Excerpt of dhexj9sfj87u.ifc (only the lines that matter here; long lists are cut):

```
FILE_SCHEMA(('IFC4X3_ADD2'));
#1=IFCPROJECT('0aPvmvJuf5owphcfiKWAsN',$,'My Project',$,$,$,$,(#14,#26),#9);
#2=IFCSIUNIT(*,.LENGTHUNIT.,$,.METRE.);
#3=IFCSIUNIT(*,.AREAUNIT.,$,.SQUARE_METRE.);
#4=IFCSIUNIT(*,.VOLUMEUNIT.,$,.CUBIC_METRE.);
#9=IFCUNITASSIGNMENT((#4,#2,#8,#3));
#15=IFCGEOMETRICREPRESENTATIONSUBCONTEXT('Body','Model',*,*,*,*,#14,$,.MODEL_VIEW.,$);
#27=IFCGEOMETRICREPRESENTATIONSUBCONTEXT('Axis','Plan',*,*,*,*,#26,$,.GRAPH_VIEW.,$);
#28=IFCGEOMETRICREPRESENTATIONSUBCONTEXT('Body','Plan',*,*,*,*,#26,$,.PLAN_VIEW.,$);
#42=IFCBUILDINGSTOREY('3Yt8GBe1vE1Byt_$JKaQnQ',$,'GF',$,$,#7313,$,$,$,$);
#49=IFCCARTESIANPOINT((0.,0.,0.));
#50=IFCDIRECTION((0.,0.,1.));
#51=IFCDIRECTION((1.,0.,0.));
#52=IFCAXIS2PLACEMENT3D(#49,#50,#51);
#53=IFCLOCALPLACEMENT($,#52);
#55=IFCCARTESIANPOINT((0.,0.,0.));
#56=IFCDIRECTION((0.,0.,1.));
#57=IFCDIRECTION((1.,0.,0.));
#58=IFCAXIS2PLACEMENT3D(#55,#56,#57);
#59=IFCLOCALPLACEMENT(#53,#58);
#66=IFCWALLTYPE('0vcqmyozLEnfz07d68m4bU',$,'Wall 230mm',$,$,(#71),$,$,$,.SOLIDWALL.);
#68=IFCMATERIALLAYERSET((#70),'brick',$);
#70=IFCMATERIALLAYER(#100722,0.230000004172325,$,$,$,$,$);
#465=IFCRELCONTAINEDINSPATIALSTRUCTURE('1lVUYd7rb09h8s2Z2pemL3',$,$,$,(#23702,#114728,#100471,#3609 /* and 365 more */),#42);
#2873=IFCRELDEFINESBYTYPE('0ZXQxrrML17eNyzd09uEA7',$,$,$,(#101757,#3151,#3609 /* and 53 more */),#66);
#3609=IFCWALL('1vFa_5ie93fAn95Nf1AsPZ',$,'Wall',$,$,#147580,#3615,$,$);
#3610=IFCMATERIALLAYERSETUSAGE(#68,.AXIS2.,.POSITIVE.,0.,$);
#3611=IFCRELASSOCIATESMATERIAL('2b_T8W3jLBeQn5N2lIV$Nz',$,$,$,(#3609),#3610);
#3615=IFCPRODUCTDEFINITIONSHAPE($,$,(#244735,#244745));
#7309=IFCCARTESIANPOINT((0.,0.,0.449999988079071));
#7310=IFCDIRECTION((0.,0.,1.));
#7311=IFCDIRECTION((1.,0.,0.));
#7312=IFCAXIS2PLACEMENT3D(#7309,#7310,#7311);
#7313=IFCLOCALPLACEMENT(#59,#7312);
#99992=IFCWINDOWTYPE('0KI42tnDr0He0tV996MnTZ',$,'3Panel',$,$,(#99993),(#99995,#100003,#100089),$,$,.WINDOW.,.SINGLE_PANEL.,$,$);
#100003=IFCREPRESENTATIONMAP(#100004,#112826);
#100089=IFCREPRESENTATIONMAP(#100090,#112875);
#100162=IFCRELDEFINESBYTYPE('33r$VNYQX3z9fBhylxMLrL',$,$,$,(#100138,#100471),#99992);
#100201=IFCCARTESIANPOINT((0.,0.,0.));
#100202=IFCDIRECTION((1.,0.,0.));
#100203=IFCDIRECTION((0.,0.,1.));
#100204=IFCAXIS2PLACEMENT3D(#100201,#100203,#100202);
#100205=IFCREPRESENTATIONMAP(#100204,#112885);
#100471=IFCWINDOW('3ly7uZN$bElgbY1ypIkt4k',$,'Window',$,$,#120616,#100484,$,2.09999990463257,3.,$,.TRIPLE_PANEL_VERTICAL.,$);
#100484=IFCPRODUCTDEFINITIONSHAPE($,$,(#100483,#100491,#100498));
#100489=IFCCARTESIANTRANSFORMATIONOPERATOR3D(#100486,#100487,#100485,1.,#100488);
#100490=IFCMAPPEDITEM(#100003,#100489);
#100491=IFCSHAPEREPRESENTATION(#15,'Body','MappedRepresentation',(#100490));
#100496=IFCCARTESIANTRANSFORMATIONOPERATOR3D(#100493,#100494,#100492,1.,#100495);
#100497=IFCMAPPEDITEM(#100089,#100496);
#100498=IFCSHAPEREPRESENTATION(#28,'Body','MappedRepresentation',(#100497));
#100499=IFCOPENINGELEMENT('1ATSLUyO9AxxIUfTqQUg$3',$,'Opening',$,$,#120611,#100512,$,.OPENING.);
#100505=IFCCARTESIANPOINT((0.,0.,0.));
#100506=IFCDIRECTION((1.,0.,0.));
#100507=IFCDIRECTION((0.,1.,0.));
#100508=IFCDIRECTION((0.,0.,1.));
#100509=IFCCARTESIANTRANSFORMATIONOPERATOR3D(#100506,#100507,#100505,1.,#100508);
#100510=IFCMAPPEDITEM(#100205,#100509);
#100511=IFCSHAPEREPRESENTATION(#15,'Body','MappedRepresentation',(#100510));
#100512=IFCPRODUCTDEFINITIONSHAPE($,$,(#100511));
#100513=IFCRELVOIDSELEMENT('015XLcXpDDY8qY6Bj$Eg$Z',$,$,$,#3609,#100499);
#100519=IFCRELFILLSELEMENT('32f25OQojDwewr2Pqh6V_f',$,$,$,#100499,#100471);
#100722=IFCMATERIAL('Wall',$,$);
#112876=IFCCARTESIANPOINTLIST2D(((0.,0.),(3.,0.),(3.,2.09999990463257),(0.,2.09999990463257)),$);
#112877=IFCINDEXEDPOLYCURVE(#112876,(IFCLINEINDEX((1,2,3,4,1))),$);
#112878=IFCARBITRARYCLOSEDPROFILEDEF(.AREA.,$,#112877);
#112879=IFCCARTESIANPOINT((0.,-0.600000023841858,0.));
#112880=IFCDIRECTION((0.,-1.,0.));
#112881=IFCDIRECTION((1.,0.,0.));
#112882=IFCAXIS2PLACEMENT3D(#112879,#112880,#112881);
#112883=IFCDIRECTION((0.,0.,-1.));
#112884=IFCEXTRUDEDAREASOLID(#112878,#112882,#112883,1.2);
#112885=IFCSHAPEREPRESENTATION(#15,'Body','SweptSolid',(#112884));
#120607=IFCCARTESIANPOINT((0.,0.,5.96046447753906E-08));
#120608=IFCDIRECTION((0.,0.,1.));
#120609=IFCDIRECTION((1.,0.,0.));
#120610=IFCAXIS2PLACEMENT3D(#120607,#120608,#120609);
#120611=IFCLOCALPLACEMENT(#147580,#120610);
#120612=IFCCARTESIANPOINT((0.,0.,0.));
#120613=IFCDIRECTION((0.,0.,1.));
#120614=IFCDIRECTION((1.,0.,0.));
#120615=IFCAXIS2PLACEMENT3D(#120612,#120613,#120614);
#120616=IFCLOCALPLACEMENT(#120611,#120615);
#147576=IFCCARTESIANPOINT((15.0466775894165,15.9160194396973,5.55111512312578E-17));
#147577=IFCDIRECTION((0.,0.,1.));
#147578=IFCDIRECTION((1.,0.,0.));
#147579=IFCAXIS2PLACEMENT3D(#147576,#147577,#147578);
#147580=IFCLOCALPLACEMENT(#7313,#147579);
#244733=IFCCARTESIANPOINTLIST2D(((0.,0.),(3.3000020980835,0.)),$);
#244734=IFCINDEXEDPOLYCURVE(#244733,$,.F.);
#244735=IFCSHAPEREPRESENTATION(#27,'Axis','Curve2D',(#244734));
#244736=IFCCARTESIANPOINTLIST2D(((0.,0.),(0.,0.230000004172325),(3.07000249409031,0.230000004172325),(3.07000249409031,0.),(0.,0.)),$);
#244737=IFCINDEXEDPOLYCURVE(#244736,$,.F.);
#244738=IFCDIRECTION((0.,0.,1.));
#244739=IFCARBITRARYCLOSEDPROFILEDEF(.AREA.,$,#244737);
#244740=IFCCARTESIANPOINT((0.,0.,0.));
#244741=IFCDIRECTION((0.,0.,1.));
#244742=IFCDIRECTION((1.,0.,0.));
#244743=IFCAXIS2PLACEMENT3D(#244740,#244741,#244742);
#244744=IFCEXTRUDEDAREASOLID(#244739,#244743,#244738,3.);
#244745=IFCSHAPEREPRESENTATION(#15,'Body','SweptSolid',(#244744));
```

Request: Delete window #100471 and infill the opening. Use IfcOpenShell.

```python
import ifcopenshell
import ifcopenshell.api.feature
import ifcopenshell.api.root
import ifcopenshell.geom
import ifcopenshell.util.shape

model = ifcopenshell.open("dhexj9sfj87u.ifc")
settings = ifcopenshell.geom.settings()


def volume(element):
    """Net volume in cubic metres, openings subtracted."""
    shape = ifcopenshell.geom.create_shape(settings, element)
    return ifcopenshell.util.shape.get_volume(shape.geometry)


window = model.by_id(100471)
opening = window.FillsVoids[0].RelatingOpeningElement
wall = opening.VoidsElements[0].RelatingBuildingElement
before = volume(wall)

ifcopenshell.api.root.remove_product(model, product=window)
ifcopenshell.api.feature.remove_feature(model, feature=opening)

after = volume(wall)

print(f"wall volume {before:.3f} -> {after:.3f} m3")

model.write("dhexj9sfj87u_updated.ifc")
```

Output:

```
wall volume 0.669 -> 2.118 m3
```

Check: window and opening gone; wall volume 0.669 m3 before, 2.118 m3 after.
